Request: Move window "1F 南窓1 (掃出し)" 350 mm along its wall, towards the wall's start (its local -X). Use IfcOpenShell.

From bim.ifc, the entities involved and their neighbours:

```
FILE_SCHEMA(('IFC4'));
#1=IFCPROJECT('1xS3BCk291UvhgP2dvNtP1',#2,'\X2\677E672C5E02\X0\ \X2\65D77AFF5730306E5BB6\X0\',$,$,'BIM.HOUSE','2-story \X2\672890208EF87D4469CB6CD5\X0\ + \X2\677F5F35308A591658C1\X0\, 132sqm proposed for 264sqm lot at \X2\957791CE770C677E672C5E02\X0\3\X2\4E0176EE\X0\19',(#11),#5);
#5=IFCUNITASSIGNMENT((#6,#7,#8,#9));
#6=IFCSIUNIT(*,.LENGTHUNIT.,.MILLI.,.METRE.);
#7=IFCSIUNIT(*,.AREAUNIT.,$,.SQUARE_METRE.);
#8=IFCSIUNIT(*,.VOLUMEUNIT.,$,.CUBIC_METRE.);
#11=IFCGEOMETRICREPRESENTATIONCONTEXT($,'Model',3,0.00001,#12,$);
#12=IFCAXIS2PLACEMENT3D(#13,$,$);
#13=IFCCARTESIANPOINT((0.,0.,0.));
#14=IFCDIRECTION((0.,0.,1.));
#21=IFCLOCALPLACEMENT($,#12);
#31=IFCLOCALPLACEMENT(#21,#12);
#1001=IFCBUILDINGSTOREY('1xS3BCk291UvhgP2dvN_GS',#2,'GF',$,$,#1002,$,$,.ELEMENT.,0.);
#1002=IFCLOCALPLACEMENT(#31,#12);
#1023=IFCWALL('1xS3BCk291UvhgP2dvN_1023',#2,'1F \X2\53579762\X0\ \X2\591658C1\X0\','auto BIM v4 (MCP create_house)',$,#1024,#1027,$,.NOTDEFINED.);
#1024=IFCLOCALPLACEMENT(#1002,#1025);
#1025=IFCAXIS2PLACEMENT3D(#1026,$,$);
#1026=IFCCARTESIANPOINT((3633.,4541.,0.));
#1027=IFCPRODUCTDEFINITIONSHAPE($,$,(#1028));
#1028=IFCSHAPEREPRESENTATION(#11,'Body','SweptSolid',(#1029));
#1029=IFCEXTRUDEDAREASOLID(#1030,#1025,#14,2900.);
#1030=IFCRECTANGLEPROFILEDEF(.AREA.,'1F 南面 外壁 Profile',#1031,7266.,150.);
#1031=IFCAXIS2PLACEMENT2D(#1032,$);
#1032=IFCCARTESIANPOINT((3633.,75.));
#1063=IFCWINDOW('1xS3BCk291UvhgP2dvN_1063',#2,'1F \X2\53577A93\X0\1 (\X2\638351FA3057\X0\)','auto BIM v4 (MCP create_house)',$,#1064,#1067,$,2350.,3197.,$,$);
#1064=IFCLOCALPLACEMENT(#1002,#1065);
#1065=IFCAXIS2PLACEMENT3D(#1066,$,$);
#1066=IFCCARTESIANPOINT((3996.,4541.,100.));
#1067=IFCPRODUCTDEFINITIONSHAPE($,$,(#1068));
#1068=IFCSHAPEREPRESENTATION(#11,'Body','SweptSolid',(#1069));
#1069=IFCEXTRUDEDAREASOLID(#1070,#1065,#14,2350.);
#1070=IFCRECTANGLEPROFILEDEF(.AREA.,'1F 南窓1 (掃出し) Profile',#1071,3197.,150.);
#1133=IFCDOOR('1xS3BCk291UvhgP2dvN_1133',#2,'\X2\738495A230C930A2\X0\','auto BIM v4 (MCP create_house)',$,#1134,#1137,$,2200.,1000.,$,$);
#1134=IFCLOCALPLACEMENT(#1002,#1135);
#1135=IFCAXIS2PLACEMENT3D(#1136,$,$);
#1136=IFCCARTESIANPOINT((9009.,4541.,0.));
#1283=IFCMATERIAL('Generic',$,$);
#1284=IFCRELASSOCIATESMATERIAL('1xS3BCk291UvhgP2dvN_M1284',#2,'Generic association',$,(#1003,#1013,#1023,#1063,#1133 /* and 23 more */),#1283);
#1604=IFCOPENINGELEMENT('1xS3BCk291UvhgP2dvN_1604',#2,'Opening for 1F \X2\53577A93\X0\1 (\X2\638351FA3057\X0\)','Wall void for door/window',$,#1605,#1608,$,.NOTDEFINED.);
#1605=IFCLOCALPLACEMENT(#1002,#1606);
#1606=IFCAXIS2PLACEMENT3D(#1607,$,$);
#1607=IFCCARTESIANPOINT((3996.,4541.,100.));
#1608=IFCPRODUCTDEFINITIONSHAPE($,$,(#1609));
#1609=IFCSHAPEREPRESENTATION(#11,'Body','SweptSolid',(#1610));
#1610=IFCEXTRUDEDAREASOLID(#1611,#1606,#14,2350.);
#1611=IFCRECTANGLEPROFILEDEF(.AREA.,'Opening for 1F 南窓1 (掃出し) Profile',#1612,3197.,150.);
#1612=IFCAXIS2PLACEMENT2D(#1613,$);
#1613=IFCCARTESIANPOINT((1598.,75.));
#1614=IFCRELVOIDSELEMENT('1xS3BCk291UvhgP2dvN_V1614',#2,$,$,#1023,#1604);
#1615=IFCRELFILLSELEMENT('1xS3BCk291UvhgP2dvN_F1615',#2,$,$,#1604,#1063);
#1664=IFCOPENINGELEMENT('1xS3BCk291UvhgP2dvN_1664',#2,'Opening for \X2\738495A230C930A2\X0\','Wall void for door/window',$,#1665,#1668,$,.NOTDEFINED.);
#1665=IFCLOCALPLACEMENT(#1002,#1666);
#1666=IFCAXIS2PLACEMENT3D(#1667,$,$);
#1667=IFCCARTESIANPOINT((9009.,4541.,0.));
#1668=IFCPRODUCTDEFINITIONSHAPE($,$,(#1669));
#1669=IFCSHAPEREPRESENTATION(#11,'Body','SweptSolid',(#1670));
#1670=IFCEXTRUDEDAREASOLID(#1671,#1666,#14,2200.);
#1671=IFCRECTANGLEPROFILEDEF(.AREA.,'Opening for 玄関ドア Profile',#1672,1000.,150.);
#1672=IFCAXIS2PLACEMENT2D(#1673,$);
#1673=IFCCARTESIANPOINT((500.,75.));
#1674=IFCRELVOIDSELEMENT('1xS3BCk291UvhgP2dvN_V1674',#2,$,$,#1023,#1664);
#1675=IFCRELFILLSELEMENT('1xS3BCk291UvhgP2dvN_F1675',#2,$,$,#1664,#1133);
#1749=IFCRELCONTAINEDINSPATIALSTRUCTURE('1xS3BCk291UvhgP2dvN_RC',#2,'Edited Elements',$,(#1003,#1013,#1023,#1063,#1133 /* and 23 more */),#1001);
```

```python
import ifcopenshell
import ifcopenshell.api.geometry
import ifcopenshell.util.placement
import ifcopenshell.util.unit

model = ifcopenshell.open("bim.ifc")
unit_scale = ifcopenshell.util.unit.calculate_unit_scale(model)

window = model.by_id(1063)
opening = window.FillsVoids[0].RelatingOpeningElement
wall = opening.VoidsElements[0].RelatingBuildingElement

wall_matrix = ifcopenshell.util.placement.get_local_placement(wall.ObjectPlacement)
shift = wall_matrix[:3, 0] * -0.35 / unit_scale
before = ifcopenshell.util.placement.get_local_placement(window.ObjectPlacement)[:3, 3].copy()

# The window is not placed relative to its opening, so move both.
for product in (opening, window):
    matrix = ifcopenshell.util.placement.get_local_placement(product.ObjectPlacement)
    matrix[:3, 3] += shift
    ifcopenshell.api.geometry.edit_object_placement(model, product=product, matrix=matrix, is_si=False)

after = ifcopenshell.util.placement.get_local_placement(window.ObjectPlacement)[:3, 3]
print("window moved by", (after - before).round(3) + 0.0)

model.write("bim_v2.ifc")
```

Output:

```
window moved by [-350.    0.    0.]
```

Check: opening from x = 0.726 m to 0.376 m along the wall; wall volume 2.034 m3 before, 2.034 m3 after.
